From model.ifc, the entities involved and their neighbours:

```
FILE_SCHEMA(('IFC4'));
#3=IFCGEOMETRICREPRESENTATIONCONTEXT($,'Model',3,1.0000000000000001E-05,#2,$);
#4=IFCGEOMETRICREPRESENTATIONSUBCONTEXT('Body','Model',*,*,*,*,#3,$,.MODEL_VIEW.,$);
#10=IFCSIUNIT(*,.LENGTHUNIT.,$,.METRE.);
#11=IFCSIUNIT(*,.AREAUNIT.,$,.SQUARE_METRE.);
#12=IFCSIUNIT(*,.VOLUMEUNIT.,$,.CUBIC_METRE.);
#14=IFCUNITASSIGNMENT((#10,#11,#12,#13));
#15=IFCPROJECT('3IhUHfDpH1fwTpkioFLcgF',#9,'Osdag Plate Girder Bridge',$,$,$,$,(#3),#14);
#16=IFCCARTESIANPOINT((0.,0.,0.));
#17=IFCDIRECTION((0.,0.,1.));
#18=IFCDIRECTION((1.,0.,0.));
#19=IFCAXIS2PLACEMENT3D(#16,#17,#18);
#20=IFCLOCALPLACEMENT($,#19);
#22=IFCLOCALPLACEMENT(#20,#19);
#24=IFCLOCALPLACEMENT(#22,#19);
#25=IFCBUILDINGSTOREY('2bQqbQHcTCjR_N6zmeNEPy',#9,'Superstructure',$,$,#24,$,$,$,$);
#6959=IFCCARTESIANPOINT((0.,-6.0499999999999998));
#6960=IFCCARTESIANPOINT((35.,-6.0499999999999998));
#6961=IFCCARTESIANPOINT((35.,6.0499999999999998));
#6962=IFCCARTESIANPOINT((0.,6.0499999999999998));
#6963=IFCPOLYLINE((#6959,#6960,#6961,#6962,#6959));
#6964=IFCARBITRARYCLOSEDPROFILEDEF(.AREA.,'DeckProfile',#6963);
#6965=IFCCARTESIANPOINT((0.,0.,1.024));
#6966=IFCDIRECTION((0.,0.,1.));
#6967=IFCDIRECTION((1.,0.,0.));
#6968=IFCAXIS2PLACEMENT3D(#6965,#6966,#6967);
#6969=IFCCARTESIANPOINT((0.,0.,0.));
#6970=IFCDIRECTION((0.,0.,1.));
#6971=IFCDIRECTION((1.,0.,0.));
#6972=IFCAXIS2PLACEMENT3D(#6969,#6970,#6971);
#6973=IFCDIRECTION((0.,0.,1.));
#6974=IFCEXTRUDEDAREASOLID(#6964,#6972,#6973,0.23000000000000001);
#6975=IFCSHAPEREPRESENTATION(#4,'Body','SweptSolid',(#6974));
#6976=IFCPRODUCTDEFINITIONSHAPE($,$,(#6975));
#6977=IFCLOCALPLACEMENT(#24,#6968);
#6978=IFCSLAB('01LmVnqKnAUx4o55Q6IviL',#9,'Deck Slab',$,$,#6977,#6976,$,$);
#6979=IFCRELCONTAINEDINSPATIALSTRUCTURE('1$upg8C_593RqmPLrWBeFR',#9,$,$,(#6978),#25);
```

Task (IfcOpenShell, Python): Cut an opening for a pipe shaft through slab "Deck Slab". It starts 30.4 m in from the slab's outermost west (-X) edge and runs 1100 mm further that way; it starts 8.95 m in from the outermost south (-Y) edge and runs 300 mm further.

```python
import numpy as np
import ifcopenshell
import ifcopenshell.api.feature
import ifcopenshell.api.geometry
import ifcopenshell.api.root
import ifcopenshell.geom
import ifcopenshell.util.placement
import ifcopenshell.util.representation
import ifcopenshell.util.shape
import ifcopenshell.util.unit

model = ifcopenshell.open("model.ifc")
unit_scale = ifcopenshell.util.unit.calculate_unit_scale(model)
settings = ifcopenshell.geom.settings()


def volume(element):
    """Net volume in cubic metres, openings subtracted."""
    shape = ifcopenshell.geom.create_shape(settings, element)
    return ifcopenshell.util.shape.get_volume(shape.geometry)


slab = model.by_id(6978)
before = volume(slab)

# Extent in the slab's own axes, in metres. The edges named are its -X and -Y sides.
slab_shape = ifcopenshell.geom.create_shape(settings, slab)
vertices = ifcopenshell.util.shape.get_vertices(slab_shape.geometry)
x_min, y_min, bottom = vertices.min(axis=0)
top = vertices[:, 2].max()

opening = ifcopenshell.api.root.create_entity(model, ifc_class="IfcOpeningElement", name="Pipe shaft opening", predefined_type="OPENING")
context = ifcopenshell.util.representation.get_context(model, "Model", "Body", "MODEL_VIEW")
width, depth = 1.1, 0.3
outline = [(0.0, 0.0), (width, 0.0), (width, depth), (0.0, depth), (0.0, 0.0)]
# Overshoot both faces by 50 mm so the cut is clean.
shape = ifcopenshell.api.geometry.add_slab_representation(
    model, context=context, depth=top - bottom + 0.1, polyline=outline
)
ifcopenshell.api.geometry.assign_representation(model, product=opening, representation=shape)

matrix = ifcopenshell.util.placement.get_local_placement(slab.ObjectPlacement)
matrix[:, 3] = matrix @ np.append(np.array([x_min + 30.4, y_min + 8.95, bottom - 0.05]) / unit_scale, 1.0)
ifcopenshell.api.geometry.edit_object_placement(model, product=opening, matrix=matrix, is_si=False)
ifcopenshell.api.feature.add_feature(model, feature=opening, element=slab)

after = volume(slab)

print(f"slab volume {before:.3f} -> {after:.3f} m3")

model.write("model-out.ifc")
```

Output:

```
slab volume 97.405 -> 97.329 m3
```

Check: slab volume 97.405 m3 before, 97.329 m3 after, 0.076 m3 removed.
